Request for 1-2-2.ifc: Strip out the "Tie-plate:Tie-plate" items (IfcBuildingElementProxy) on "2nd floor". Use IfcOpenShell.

First a look at what the model holds.

```python
import ifcopenshell
import ifcopenshell.util.element

model = ifcopenshell.open("1-2-2.ifc")
print(model.schema)
storey = next(s for s in model.by_type("IfcBuildingStorey") if s.Name == "2nd floor")
proxies = [e for e in ifcopenshell.util.element.get_decomposition(storey) if e.is_a("IfcBuildingElementProxy")]
seen = {}
for e in proxies:
    element_type = ifcopenshell.util.element.get_type(e)
    name = element_type.Name if element_type not in (None, e) else None
    seen[name] = seen.get(name, 0) + 1
for name, count in sorted(seen.items(), key=str):
    print(count, "x", name)
```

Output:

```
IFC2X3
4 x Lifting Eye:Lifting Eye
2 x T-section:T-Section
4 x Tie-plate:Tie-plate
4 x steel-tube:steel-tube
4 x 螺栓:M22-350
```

```python
import ifcopenshell
import ifcopenshell.api.root
import ifcopenshell.util.element

model = ifcopenshell.open("1-2-2.ifc")

storey = next(s for s in model.by_type("IfcBuildingStorey") if s.Name == "2nd floor")
proxies = [e for e in ifcopenshell.util.element.get_decomposition(storey) if e.is_a("IfcBuildingElementProxy")]
targets = [e for e in proxies if (t := ifcopenshell.util.element.get_type(e)) not in (None, e) and t.Name == "Tie-plate:Tie-plate"]

for e in targets:
    ifcopenshell.api.root.remove_product(model, product=e)
print(len(targets), "removed")

model.write("1-2-2_rev.ifc")
```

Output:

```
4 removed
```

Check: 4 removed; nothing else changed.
